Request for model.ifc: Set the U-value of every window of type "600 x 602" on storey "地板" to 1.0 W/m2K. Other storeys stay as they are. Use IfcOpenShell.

First a look at what the model holds.

```python
import ifcopenshell
import ifcopenshell.util.element

model = ifcopenshell.open("model.ifc")
print(model.schema)
storey = next(s for s in model.by_type("IfcBuildingStorey") if s.Name == "地板")
windows = [e for e in ifcopenshell.util.element.get_decomposition(storey) if e.is_a("IfcWindow")]
seen = {}
for e in windows:
    element_type = ifcopenshell.util.element.get_type(e)
    key = (element_type.Name if element_type != e and element_type else None, ifcopenshell.util.element.get_pset(e, "Pset_WindowCommon", "ThermalTransmittance"))
    seen[key] = seen.get(key, 0) + 1
for (name, value), count in sorted(seen.items(), key=str):
    print(count, "x", name, "|", value)
```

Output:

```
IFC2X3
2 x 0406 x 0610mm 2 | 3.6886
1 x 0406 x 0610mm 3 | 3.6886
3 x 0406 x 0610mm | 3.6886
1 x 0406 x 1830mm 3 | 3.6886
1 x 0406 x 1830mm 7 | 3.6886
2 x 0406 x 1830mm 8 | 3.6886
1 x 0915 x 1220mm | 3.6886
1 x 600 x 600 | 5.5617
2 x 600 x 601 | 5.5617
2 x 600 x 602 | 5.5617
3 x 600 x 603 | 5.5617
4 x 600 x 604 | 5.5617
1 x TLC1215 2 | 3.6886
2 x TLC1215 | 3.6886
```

```python
import ifcopenshell
import ifcopenshell.api.pset
import ifcopenshell.util.element

model = ifcopenshell.open("model.ifc")

storey = next(s for s in model.by_type("IfcBuildingStorey") if s.Name == "地板")
windows = [e for e in ifcopenshell.util.element.get_decomposition(storey) if e.is_a("IfcWindow")]

count = 0
for e in windows:
    element_type = ifcopenshell.util.element.get_type(e)
    if element_type in (None, e) or element_type.Name != "600 x 602":
        continue
    # add_pset returns the element's existing set when there is one.
    pset = ifcopenshell.api.pset.add_pset(model, product=e, name="Pset_WindowCommon")
    ifcopenshell.api.pset.edit_pset(model, pset=pset, properties={"ThermalTransmittance": 1.0})
    count += 1

print(count, "windows updated")

model.write("model_rev.ifc")
```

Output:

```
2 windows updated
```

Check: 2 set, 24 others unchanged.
